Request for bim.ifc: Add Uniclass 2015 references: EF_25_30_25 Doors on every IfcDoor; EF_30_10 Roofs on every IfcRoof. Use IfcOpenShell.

First a look at what the model holds.

```python
import ifcopenshell

model = ifcopenshell.open("bim.ifc")
print(model.schema)
print("classifications:", [c.Name for c in model.by_type("IfcClassification")])
for ifc_class in ("IfcDoor", "IfcRoof", "IfcStair", "IfcWall", "IfcWindow"):
    print(ifc_class, len(model.by_type(ifc_class)))
```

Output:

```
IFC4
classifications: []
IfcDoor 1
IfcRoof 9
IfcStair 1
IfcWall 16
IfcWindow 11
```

```python
import ifcopenshell
import ifcopenshell.api.classification

model = ifcopenshell.open("bim.ifc")

system = ifcopenshell.api.classification.add_classification(model, classification="Uniclass 2015")

codes = {
    "IfcDoor": ("EF_25_30_25", "Doors"),
    "IfcRoof": ("EF_30_10", "Roofs"),
}
for ifc_class, (code, name) in codes.items():
    products = model.by_type(ifc_class)
    ifcopenshell.api.classification.add_reference(
        model, products=products, classification=system, identification=code, name=name
    )
    print(code, len(products))

model.write("bim_v2.ifc")
```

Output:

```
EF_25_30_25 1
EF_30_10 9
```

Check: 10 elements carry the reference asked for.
